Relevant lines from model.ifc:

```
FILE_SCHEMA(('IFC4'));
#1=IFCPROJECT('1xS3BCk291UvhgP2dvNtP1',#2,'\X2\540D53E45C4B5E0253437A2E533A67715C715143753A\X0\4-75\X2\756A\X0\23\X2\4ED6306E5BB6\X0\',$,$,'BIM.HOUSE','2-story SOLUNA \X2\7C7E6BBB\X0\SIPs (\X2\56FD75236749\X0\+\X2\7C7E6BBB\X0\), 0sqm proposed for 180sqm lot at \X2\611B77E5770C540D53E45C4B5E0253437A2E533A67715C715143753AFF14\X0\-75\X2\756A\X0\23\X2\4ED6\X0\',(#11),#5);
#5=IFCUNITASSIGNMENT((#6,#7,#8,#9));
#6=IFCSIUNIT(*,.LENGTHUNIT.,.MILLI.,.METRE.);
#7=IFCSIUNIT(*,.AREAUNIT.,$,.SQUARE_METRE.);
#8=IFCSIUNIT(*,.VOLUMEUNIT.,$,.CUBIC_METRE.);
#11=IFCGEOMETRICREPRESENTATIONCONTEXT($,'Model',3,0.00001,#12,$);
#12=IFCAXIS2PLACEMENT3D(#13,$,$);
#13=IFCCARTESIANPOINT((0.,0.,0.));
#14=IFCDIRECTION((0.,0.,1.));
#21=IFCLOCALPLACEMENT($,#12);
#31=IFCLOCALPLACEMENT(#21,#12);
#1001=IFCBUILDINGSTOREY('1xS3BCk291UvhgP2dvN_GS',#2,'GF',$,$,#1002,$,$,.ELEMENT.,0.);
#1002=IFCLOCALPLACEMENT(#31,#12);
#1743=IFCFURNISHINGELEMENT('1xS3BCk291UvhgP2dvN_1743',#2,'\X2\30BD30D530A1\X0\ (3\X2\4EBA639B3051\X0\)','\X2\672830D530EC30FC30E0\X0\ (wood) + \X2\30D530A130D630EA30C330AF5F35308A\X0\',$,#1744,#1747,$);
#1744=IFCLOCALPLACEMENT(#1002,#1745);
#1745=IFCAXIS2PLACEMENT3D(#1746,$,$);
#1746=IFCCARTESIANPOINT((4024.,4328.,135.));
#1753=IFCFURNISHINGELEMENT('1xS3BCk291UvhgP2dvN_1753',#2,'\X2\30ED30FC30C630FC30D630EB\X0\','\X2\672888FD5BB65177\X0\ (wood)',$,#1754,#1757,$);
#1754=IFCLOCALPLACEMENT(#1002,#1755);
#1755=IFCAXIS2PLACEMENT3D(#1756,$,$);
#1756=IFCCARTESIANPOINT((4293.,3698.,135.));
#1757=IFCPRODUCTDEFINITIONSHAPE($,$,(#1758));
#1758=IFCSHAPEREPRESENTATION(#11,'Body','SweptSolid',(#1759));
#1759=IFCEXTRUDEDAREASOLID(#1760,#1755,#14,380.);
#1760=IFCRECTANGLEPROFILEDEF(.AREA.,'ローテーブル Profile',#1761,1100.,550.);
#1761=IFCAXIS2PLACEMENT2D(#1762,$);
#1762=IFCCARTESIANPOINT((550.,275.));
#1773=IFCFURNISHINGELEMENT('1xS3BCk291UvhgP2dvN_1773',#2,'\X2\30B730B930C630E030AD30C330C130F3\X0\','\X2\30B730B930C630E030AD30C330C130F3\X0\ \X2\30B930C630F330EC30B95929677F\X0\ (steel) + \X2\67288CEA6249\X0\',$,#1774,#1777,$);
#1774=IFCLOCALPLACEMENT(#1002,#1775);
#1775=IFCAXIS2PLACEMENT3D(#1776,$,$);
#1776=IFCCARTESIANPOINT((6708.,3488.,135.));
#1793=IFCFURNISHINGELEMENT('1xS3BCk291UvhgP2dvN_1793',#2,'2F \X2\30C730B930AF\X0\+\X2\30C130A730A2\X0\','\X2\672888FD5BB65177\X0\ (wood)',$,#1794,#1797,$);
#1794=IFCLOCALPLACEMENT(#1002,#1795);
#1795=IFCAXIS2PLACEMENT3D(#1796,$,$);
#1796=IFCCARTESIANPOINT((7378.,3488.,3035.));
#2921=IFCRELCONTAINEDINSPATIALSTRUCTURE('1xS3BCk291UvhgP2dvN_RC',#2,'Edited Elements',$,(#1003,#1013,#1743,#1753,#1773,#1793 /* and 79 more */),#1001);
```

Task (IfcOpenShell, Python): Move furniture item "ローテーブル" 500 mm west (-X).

```python
import ifcopenshell
import ifcopenshell.api.geometry
import ifcopenshell.util.placement
import ifcopenshell.util.unit

model = ifcopenshell.open("model.ifc")
unit_scale = ifcopenshell.util.unit.calculate_unit_scale(model)

item = model.by_id(1753)
matrix = ifcopenshell.util.placement.get_local_placement(item.ObjectPlacement)
matrix[0, 3] -= 0.5 / unit_scale
ifcopenshell.api.geometry.edit_object_placement(model, product=item, matrix=matrix, is_si=False)

print(ifcopenshell.util.placement.get_local_placement(item.ObjectPlacement).round(3) + 0.0)

model.write("model_rev.ifc")
```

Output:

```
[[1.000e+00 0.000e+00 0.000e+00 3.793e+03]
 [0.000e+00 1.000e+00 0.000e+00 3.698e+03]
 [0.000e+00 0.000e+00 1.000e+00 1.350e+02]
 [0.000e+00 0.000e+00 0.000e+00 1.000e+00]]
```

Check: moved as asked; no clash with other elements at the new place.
